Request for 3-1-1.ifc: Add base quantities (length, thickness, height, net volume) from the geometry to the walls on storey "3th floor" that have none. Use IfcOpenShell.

First a look at what the model holds.

```python
import ifcopenshell
import ifcopenshell.util.element
import ifcopenshell.util.unit

model = ifcopenshell.open("3-1-1.ifc")
print(model.schema)
for unit_type in ("LENGTHUNIT", "AREAUNIT", "VOLUMEUNIT"):
    print(unit_type, ifcopenshell.util.unit.calculate_unit_scale(model, unit_type))
storey = next(s for s in model.by_type("IfcBuildingStorey") if s.Name == "3th floor")
walls = [e for e in ifcopenshell.util.element.get_decomposition(storey) if e.is_a("IfcWall")]
for e in sorted(walls, key=lambda e: e.id()):
    print(e.id(), e.is_a(), e.Name, list(ifcopenshell.util.element.get_psets(e, qtos_only=True)), sep=" | ")
```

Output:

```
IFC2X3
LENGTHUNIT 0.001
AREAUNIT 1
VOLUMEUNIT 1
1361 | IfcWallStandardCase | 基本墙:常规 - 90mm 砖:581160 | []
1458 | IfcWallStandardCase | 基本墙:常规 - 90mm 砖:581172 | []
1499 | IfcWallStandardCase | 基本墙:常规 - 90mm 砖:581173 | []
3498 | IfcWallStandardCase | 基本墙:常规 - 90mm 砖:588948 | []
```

```python
import ifcopenshell
import ifcopenshell.api.pset
import ifcopenshell.geom
import ifcopenshell.util.element
import ifcopenshell.util.shape
import ifcopenshell.util.unit

model = ifcopenshell.open("3-1-1.ifc")
unit_scale = ifcopenshell.util.unit.calculate_unit_scale(model)
volume_scale = ifcopenshell.util.unit.calculate_unit_scale(model, "VOLUMEUNIT")
settings = ifcopenshell.geom.settings()

storey = next(s for s in model.by_type("IfcBuildingStorey") if s.Name == "3th floor")
walls = [e for e in ifcopenshell.util.element.get_decomposition(storey) if e.is_a("IfcWall")]

for e in sorted(walls, key=lambda e: e.id()):
    if ifcopenshell.util.element.get_psets(e, qtos_only=True, should_inherit=False):
        continue
    # Geometry comes back in metres, in the element's own axes.
    shape = ifcopenshell.geom.create_shape(settings, e)
    values = {
        "Length": ifcopenshell.util.shape.get_x(shape.geometry) / unit_scale,
        "Width": ifcopenshell.util.shape.get_y(shape.geometry) / unit_scale,
        "Height": ifcopenshell.util.shape.get_z(shape.geometry) / unit_scale,
        "NetVolume": ifcopenshell.util.shape.get_volume(shape.geometry) / volume_scale,
    }
    qto = ifcopenshell.api.pset.add_qto(model, product=e, name="BaseQuantities")
    ifcopenshell.api.pset.edit_qto(model, qto=qto, properties=values)
    print(e.id(), {k: round(v, 3) for k, v in values.items()})

model.write("3-1-1_rev.ifc")
```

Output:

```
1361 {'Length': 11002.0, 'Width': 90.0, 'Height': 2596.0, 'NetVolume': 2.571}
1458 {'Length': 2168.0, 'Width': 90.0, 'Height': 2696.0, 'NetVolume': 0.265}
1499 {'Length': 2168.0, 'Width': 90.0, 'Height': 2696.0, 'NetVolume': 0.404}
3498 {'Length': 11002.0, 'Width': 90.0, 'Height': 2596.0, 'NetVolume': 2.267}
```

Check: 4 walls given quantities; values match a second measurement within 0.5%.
